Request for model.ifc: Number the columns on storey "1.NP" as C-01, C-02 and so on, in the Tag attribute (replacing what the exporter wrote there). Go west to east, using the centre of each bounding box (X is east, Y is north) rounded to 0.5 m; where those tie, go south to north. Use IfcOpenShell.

First a look at what the model holds.

```python
import ifcopenshell
import ifcopenshell.util.element
import ifcopenshell.util.placement

model = ifcopenshell.open("model.ifc")
print(model.schema)
storey = next(s for s in model.by_type("IfcBuildingStorey") if s.Name == "1.NP")
columns = [e for e in ifcopenshell.util.element.get_decomposition(storey) if e.is_a("IfcColumn")]
for e in sorted(columns, key=lambda e: e.id()):
    origin = ifcopenshell.util.placement.get_local_placement(e.ObjectPlacement)[:3, 3]
    print(e.id(), e.Tag, e.Name, origin.round(2) + 0.0, sep=" | ")
```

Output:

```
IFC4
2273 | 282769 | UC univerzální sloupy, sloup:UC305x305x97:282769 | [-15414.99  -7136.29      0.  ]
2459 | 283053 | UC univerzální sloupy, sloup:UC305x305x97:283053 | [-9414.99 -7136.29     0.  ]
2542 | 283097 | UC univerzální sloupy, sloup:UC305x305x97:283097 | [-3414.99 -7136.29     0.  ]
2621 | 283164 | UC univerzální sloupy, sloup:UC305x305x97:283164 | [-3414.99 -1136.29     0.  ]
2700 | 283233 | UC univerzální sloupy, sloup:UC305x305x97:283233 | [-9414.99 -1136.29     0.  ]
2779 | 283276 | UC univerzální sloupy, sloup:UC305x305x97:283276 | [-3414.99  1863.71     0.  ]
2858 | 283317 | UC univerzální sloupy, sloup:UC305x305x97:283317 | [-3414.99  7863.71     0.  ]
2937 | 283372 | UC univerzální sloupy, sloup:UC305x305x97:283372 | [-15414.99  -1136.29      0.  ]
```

```python
import ifcopenshell
import ifcopenshell.geom
import ifcopenshell.util.element
import ifcopenshell.util.shape

model = ifcopenshell.open("model.ifc")
settings = ifcopenshell.geom.settings()
settings.set("use-world-coords", True)


def centre(element):
    shape = ifcopenshell.geom.create_shape(settings, element)
    return ifcopenshell.util.shape.get_bbox_centroid(shape.geometry)


storey = next(s for s in model.by_type("IfcBuildingStorey") if s.Name == "1.NP")
columns = [e for e in ifcopenshell.util.element.get_decomposition(storey) if e.is_a("IfcColumn")]

# Insertion points can sit at a corner or the storey origin, so sort by the geometry (in metres).
centres = {e: centre(e) for e in columns}
columns.sort(key=lambda e: (round(centres[e][0] / 0.5), centres[e][1]))

for i, e in enumerate(columns, start=1):
    number = f"C-{i:02d}"
    e.Tag = number
    print(e.id(), number)

model.write("model-out.ifc")
```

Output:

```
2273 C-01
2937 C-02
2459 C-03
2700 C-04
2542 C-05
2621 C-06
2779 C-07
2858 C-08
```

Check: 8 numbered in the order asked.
